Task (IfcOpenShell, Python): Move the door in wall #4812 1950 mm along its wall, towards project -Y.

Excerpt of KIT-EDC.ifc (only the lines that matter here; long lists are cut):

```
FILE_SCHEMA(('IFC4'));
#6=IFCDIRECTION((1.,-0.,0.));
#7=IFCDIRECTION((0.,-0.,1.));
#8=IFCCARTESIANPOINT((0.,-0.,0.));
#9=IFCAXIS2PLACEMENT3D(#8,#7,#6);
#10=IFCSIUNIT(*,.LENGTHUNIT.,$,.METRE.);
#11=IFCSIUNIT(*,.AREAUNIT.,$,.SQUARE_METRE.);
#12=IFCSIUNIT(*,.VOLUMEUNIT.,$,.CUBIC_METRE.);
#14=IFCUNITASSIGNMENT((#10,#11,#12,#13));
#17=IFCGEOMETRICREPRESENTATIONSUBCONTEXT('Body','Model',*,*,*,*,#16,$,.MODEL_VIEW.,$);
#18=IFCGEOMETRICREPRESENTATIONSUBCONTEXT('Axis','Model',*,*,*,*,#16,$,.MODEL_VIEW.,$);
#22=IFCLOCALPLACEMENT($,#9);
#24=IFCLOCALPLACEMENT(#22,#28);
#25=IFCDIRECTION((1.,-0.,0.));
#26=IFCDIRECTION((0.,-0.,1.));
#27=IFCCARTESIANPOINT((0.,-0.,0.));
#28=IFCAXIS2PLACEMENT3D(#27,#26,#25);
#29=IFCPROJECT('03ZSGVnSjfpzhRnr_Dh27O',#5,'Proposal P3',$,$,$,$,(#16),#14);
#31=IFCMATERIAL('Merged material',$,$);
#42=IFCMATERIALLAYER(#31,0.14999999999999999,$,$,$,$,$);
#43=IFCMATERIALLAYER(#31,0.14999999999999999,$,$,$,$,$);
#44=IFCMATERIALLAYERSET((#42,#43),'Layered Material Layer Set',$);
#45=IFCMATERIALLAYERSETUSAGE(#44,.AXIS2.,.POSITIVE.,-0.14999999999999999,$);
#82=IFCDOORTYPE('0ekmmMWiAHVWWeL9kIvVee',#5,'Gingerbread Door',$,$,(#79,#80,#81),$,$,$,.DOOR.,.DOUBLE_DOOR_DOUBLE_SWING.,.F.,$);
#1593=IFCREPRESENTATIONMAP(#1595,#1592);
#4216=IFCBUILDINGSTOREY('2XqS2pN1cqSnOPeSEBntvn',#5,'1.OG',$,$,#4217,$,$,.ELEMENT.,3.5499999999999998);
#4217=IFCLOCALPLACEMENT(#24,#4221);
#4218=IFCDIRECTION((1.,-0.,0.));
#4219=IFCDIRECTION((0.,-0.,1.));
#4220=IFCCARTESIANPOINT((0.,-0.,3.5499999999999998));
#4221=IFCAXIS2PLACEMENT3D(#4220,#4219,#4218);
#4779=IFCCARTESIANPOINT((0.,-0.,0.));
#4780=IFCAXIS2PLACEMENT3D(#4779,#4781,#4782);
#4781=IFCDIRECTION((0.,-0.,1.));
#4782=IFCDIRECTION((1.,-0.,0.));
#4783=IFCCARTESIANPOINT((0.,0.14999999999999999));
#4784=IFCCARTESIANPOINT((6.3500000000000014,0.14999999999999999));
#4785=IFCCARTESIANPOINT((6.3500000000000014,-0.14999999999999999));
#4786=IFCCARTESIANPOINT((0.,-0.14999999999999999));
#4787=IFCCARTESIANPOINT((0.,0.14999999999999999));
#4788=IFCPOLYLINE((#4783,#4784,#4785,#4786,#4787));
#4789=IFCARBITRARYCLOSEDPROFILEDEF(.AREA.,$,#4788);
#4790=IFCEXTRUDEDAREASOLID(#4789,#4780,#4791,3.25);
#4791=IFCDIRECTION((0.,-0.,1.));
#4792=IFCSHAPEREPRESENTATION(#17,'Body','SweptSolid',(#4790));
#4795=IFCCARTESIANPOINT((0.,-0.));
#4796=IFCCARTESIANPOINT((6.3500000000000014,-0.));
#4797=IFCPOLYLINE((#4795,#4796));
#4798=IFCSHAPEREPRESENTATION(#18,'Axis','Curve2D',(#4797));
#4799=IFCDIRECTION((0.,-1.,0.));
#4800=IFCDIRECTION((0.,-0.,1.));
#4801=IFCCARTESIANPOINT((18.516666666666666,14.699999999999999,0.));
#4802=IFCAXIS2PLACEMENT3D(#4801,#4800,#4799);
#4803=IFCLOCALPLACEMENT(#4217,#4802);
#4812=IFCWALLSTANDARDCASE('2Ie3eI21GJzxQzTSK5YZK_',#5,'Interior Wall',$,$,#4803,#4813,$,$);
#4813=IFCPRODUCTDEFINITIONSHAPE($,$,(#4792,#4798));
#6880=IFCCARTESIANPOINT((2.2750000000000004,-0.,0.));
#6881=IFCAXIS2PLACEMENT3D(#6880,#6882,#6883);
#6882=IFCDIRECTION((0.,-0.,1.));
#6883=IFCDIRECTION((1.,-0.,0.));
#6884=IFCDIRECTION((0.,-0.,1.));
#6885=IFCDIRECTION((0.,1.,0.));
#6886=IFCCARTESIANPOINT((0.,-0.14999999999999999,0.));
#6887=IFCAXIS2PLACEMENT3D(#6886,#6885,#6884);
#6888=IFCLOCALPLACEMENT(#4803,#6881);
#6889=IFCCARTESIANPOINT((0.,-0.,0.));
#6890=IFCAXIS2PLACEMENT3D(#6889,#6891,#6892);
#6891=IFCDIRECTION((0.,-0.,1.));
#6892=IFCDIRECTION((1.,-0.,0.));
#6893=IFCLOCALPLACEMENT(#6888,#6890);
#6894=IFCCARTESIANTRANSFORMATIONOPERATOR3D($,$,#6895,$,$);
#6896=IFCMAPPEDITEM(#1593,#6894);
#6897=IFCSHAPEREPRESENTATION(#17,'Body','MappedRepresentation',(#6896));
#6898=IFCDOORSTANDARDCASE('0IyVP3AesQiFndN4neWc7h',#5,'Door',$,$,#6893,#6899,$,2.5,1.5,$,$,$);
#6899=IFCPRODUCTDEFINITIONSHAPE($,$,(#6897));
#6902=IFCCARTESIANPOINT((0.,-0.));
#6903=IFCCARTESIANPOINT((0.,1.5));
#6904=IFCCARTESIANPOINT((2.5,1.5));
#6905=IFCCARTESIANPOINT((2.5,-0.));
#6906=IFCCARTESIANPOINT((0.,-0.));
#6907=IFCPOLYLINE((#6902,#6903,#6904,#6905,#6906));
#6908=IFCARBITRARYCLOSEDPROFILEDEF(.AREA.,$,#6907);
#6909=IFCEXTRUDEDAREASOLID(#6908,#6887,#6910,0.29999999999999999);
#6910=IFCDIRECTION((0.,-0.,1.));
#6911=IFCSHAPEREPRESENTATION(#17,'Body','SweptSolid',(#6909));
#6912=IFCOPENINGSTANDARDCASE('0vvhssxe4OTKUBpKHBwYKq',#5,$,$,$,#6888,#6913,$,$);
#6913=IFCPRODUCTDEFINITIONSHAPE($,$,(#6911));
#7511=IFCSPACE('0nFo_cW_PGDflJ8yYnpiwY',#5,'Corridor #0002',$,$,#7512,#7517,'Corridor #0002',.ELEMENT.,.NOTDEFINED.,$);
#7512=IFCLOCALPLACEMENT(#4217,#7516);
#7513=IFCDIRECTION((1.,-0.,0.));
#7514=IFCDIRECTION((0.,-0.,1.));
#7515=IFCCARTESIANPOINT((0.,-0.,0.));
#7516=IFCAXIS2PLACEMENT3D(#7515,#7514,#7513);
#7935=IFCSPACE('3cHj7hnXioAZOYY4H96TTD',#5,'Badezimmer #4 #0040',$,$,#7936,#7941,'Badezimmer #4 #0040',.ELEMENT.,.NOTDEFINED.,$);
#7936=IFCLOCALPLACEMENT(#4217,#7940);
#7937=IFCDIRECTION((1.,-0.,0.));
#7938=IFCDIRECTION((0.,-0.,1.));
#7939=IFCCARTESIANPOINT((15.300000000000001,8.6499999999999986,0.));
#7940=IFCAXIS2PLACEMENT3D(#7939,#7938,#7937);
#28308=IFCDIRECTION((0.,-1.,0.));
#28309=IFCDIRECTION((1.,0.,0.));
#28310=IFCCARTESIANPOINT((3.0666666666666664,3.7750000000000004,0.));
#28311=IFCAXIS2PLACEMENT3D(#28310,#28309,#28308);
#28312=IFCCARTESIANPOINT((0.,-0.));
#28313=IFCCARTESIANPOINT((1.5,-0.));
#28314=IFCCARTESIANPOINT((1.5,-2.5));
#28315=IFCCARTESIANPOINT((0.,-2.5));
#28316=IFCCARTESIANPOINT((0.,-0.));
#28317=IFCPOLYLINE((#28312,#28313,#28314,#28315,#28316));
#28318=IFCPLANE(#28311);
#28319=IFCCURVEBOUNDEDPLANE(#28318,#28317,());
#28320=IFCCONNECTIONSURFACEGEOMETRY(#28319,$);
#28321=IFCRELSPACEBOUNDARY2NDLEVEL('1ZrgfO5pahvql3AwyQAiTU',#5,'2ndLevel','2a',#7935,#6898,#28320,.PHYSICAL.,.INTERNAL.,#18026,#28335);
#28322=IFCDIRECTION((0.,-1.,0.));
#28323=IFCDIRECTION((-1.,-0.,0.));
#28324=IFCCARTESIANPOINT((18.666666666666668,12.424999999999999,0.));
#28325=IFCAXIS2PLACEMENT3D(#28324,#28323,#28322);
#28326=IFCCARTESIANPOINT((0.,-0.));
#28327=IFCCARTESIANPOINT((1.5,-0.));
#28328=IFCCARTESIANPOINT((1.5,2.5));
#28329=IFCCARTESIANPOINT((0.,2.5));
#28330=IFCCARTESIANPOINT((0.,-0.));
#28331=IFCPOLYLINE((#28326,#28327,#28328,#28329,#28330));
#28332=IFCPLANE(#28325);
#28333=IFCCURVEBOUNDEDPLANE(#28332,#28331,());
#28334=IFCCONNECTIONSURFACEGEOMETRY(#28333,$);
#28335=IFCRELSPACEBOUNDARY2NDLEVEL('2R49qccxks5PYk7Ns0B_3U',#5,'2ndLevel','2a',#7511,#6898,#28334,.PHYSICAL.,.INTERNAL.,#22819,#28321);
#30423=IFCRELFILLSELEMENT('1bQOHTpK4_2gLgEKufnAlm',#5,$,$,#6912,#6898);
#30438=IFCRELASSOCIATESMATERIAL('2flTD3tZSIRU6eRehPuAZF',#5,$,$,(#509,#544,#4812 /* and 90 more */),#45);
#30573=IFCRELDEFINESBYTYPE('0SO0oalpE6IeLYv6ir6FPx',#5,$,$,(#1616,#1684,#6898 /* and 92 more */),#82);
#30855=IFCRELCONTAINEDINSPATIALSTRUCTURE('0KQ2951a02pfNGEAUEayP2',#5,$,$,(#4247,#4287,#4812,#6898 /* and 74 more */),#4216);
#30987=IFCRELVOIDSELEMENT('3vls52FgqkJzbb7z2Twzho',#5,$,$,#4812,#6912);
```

```python
import numpy as np
import ifcopenshell
import ifcopenshell.api.geometry
import ifcopenshell.util.placement
import ifcopenshell.util.unit

model = ifcopenshell.open("KIT-EDC.ifc")
unit_scale = ifcopenshell.util.unit.calculate_unit_scale(model)

door = model.by_id(6898)
opening = door.FillsVoids[0].RelatingOpeningElement
wall = opening.VoidsElements[0].RelatingBuildingElement

wall_matrix = ifcopenshell.util.placement.get_local_placement(wall.ObjectPlacement)
shift = wall_matrix[:3, 0] * 1.95 / unit_scale
before = ifcopenshell.util.placement.get_local_placement(door.ObjectPlacement)[:3, 3].copy()

# The door is placed relative to its opening, so it follows when the opening moves.
matrix = ifcopenshell.util.placement.get_local_placement(opening.ObjectPlacement)
matrix[:3, 3] += shift
ifcopenshell.api.geometry.edit_object_placement(
    model, product=opening, matrix=matrix, is_si=False, should_transform_children=True
)

# Space boundary surfaces are stored in each space's coordinates; move them too.
for rel in door.ProvidesBoundaries:
    if not rel.ConnectionGeometry:
        continue
    surface = rel.ConnectionGeometry.SurfaceOnRelatingElement.BasisSurface
    space_matrix = ifcopenshell.util.placement.get_local_placement(rel.RelatingSpace.ObjectPlacement)
    point = np.array(surface.Position.Location.Coordinates) + space_matrix[:3, :3].T @ shift
    surface.Position = model.createIfcAxis2Placement3D(
        model.createIfcCartesianPoint(point.tolist()), surface.Position.Axis, surface.Position.RefDirection
    )

after = ifcopenshell.util.placement.get_local_placement(door.ObjectPlacement)[:3, 3]
print("door moved by", (after - before).round(3) + 0.0)

model.write("KIT-EDC_rev.ifc")
```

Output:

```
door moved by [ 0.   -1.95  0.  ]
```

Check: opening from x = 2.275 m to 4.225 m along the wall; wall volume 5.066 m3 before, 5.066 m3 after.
